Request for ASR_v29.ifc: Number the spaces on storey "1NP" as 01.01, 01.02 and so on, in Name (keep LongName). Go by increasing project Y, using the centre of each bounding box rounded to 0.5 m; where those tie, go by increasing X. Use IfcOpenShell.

First a look at what the model holds.

```python
import ifcopenshell
import ifcopenshell.util.element
import ifcopenshell.util.placement

model = ifcopenshell.open("ASR_v29.ifc")
print(model.schema)
storey = next(s for s in model.by_type("IfcBuildingStorey") if s.Name == "1NP")
spaces = [e for e in ifcopenshell.util.element.get_decomposition(storey) if e.is_a("IfcSpace")]
for e in sorted(spaces, key=lambda e: e.id()):
    origin = ifcopenshell.util.placement.get_local_placement(e.ObjectPlacement)[:3, 3]
    print(e.id(), e.Name, e.LongName, origin.round(2) + 0.0, sep=" | ")
```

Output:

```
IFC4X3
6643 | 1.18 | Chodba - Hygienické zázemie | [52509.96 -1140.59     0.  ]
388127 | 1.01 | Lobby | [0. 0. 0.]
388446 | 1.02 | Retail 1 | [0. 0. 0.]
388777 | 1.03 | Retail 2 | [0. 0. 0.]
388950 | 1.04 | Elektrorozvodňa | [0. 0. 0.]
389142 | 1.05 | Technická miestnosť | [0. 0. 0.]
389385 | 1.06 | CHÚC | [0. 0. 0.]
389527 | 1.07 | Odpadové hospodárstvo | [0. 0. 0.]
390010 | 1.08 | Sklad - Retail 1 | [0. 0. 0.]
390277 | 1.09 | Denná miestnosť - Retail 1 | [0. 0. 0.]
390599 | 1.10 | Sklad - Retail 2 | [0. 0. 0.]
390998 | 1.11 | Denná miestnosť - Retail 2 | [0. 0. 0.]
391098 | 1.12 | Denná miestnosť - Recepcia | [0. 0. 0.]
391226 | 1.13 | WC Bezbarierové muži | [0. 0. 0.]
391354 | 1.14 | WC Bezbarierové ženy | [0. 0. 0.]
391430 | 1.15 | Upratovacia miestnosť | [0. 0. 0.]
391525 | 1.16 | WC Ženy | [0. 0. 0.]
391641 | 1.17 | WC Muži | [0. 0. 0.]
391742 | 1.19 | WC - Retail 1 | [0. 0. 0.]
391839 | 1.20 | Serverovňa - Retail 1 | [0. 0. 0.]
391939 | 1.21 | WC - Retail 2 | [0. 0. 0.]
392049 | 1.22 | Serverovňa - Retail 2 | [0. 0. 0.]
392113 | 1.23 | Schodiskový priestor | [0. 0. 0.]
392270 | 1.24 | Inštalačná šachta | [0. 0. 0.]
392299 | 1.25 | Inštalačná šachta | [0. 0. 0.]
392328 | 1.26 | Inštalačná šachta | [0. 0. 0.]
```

```python
import ifcopenshell
import ifcopenshell.geom
import ifcopenshell.util.element
import ifcopenshell.util.shape

model = ifcopenshell.open("ASR_v29.ifc")
settings = ifcopenshell.geom.settings()
settings.set("use-world-coords", True)


def centre(element):
    shape = ifcopenshell.geom.create_shape(settings, element)
    return ifcopenshell.util.shape.get_bbox_centroid(shape.geometry)


storey = next(s for s in model.by_type("IfcBuildingStorey") if s.Name == "1NP")
spaces = [e for e in ifcopenshell.util.element.get_decomposition(storey) if e.is_a("IfcSpace")]

# Insertion points can sit at a corner or the storey origin, so sort by the geometry (in metres).
centres = {e: centre(e) for e in spaces}
spaces.sort(key=lambda e: (round(centres[e][1] / 0.5), centres[e][0]))

for i, e in enumerate(spaces, start=1):
    number = f"01.{i:02d}"
    e.Name = number
    print(e.id(), number)

model.write("ASR_v29_v2.ifc")
```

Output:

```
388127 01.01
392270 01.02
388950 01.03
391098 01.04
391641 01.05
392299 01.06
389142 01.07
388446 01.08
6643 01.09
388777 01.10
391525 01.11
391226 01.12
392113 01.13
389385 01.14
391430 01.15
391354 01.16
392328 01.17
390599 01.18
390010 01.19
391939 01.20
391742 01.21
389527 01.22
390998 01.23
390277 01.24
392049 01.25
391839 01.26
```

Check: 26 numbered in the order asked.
